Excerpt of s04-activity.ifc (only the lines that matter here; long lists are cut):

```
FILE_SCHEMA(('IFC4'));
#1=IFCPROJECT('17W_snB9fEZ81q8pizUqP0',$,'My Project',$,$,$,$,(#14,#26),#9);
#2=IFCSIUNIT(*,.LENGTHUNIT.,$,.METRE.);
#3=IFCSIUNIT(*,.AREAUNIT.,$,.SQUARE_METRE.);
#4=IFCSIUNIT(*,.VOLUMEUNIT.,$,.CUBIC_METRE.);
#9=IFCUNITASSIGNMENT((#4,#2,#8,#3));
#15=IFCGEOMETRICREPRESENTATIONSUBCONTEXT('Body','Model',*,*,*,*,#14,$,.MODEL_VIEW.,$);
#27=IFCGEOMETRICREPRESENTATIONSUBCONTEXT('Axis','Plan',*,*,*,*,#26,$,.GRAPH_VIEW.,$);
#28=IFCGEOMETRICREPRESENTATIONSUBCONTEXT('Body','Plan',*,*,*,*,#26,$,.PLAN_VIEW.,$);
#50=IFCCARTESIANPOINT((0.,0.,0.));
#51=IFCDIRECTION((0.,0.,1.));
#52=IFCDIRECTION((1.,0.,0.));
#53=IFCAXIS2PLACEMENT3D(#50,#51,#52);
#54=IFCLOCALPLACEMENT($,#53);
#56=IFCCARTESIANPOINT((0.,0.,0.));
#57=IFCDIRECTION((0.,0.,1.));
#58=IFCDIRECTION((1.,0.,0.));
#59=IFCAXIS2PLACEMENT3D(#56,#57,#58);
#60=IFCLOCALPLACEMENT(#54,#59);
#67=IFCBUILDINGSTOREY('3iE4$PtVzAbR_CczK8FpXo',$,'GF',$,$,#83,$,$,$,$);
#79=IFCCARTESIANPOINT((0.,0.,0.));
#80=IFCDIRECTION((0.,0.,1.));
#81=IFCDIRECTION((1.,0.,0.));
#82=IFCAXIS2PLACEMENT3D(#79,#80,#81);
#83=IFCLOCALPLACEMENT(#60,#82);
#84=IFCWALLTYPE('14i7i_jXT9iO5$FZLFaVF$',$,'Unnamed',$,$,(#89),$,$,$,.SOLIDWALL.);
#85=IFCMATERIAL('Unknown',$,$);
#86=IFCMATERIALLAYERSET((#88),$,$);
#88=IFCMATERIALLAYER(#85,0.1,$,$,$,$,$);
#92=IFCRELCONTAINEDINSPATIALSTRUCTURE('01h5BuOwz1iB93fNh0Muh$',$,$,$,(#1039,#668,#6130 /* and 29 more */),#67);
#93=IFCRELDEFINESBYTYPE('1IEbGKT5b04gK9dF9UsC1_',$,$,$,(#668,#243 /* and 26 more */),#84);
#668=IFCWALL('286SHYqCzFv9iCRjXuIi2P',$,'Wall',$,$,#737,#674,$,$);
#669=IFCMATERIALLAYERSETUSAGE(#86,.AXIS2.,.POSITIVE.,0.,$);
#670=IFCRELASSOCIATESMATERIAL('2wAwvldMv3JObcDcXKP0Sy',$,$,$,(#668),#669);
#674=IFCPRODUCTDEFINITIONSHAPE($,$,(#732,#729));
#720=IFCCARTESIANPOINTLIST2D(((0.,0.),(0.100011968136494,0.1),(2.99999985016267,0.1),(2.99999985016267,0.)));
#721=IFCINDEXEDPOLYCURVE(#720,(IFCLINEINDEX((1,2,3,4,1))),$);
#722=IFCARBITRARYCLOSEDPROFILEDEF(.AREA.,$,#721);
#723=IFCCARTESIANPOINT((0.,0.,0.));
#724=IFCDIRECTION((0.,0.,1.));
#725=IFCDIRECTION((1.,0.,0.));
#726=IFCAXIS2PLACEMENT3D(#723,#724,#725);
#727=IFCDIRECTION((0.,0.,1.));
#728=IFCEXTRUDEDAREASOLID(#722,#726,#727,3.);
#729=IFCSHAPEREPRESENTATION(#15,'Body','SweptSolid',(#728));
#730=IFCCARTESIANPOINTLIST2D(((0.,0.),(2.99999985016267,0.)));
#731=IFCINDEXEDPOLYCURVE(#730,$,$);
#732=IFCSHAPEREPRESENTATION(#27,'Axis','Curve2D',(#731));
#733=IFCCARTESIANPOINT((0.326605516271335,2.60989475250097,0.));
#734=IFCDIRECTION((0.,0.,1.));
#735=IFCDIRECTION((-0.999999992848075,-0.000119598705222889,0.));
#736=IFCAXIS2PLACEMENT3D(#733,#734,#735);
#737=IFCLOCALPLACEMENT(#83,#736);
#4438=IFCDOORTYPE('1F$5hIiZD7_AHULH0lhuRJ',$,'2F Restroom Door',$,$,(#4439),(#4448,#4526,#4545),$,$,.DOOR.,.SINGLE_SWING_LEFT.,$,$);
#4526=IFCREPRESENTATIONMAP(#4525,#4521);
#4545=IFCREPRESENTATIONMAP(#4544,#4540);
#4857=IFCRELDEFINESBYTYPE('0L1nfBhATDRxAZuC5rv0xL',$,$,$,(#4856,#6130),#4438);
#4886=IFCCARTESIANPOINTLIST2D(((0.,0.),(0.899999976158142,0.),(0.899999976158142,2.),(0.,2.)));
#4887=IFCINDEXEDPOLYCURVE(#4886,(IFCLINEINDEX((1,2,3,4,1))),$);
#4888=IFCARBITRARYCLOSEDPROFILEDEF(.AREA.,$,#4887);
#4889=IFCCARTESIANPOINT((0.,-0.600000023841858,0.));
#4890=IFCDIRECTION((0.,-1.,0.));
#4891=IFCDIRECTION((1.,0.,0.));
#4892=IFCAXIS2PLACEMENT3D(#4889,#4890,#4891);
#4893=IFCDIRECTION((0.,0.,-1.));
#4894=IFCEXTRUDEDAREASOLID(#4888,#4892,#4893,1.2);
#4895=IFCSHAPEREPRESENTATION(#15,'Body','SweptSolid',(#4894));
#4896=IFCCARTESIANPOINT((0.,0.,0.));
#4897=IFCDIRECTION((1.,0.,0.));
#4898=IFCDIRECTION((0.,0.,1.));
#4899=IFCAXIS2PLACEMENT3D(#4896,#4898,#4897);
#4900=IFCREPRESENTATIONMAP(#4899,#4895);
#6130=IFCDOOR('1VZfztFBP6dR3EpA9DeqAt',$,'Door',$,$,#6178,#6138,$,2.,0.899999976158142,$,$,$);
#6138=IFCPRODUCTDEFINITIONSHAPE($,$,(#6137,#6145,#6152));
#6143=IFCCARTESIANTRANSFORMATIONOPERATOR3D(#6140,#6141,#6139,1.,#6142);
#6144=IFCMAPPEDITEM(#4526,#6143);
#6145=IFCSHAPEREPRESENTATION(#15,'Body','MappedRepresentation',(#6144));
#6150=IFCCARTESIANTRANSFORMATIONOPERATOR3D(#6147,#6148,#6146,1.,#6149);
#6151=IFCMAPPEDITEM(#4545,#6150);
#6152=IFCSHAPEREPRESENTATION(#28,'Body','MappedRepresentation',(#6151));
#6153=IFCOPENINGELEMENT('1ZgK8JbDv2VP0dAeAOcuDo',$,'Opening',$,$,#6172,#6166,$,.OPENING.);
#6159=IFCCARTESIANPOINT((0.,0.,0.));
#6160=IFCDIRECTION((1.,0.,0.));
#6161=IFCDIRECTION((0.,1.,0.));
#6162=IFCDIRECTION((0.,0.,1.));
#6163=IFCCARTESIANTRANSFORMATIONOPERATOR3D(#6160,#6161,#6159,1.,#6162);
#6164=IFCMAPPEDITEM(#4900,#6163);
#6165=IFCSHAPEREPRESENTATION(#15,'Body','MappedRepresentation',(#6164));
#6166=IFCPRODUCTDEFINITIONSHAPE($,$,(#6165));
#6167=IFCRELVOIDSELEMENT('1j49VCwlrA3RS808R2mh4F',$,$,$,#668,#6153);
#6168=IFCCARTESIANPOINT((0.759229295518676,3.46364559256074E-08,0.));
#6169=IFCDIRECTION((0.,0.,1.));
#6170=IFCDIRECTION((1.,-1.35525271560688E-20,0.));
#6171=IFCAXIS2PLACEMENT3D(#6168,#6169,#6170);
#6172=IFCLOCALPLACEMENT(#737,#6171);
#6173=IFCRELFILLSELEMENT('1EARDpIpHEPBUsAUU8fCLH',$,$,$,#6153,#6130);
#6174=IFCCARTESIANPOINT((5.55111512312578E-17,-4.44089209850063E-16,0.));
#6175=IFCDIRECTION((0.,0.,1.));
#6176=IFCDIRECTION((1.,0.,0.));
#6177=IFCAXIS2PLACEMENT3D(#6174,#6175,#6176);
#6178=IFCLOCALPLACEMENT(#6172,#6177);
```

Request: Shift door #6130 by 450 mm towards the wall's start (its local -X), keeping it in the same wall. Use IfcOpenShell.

```python
import ifcopenshell
import ifcopenshell.api.geometry
import ifcopenshell.util.placement
import ifcopenshell.util.unit

model = ifcopenshell.open("s04-activity.ifc")
unit_scale = ifcopenshell.util.unit.calculate_unit_scale(model)

door = model.by_id(6130)
opening = door.FillsVoids[0].RelatingOpeningElement
wall = opening.VoidsElements[0].RelatingBuildingElement

wall_matrix = ifcopenshell.util.placement.get_local_placement(wall.ObjectPlacement)
shift = wall_matrix[:3, 0] * -0.45 / unit_scale
before = ifcopenshell.util.placement.get_local_placement(door.ObjectPlacement)[:3, 3].copy()

# The door is placed relative to its opening, so it follows when the opening moves.
matrix = ifcopenshell.util.placement.get_local_placement(opening.ObjectPlacement)
matrix[:3, 3] += shift
ifcopenshell.api.geometry.edit_object_placement(
    model, product=opening, matrix=matrix, is_si=False, should_transform_children=True
)

after = ifcopenshell.util.placement.get_local_placement(door.ObjectPlacement)[:3, 3]
print("door moved by", (after - before).round(3) + 0.0)

model.write("s04-activity_updated.ifc")
```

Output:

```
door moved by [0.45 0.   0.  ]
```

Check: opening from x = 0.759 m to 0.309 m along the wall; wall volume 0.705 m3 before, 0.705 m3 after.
